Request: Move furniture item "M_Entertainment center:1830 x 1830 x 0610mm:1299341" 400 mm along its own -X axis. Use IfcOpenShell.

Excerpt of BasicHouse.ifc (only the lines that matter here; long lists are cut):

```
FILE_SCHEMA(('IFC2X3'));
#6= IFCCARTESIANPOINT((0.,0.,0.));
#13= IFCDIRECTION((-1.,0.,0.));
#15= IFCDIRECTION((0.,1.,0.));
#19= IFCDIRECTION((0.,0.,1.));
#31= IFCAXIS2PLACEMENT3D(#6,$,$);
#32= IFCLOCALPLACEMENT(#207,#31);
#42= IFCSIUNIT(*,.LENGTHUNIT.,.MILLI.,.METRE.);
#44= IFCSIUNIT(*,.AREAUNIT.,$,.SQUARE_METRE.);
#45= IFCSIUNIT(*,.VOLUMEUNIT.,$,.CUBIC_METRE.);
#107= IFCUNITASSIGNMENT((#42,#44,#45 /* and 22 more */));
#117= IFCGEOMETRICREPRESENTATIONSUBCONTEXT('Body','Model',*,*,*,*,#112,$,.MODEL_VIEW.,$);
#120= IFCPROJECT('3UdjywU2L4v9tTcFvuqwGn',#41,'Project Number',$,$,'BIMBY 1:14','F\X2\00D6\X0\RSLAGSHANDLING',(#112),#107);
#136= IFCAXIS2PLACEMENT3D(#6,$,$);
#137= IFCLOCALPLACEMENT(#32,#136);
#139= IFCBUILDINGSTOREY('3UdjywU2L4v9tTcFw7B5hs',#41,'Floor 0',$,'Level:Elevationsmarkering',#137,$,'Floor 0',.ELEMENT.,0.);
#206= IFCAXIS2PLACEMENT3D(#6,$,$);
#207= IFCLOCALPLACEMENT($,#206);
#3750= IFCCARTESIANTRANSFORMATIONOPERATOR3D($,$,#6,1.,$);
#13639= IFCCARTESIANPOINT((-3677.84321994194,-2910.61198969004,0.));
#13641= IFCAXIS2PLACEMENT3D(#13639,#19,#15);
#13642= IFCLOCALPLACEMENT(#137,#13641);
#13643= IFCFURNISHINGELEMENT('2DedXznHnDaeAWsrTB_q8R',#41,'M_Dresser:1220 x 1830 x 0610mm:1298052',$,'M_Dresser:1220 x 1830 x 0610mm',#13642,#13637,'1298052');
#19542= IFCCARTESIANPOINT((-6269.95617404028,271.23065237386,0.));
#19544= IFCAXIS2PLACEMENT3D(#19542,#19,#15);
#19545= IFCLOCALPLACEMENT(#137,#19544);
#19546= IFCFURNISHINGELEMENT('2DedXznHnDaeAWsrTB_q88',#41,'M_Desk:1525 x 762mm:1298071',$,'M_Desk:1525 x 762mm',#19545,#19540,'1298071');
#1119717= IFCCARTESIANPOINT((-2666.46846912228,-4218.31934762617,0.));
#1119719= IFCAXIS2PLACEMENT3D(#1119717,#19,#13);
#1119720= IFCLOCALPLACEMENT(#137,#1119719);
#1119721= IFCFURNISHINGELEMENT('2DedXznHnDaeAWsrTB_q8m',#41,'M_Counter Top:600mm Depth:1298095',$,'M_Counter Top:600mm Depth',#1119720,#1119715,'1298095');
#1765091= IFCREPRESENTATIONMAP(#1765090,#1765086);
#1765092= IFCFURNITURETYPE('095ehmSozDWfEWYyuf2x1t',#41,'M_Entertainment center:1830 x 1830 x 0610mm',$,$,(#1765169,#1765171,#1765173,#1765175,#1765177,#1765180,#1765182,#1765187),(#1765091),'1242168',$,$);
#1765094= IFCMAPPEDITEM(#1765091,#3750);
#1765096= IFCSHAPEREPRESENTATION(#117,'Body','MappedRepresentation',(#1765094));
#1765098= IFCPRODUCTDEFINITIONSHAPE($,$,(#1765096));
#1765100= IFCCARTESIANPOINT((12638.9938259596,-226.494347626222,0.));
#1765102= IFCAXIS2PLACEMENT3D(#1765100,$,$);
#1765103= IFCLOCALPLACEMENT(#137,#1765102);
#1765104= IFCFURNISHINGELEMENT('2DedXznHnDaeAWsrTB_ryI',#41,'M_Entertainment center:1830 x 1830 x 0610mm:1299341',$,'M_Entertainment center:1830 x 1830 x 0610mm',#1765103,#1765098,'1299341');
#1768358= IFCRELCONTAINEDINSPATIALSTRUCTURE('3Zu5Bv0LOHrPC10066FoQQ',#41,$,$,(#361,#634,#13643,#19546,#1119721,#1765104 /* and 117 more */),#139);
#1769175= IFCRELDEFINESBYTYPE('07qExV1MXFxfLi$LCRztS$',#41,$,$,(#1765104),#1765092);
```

```python
import ifcopenshell
import ifcopenshell.api.geometry
import ifcopenshell.util.placement
import ifcopenshell.util.unit

model = ifcopenshell.open("BasicHouse.ifc")
unit_scale = ifcopenshell.util.unit.calculate_unit_scale(model)

item = model.by_guid("2DedXznHnDaeAWsrTB_ryI")
matrix = ifcopenshell.util.placement.get_local_placement(item.ObjectPlacement)
matrix[:3, 3] -= matrix[:3, 0] * 0.4 / unit_scale
ifcopenshell.api.geometry.edit_object_placement(model, product=item, matrix=matrix, is_si=False)

print(ifcopenshell.util.placement.get_local_placement(item.ObjectPlacement).round(3) + 0.0)

model.write("BasicHouse_rev.ifc")
```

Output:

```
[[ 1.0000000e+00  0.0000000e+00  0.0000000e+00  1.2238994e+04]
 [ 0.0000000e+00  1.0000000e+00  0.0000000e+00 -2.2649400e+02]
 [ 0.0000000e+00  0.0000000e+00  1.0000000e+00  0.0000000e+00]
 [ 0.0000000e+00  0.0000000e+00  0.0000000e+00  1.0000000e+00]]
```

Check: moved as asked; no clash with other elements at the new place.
